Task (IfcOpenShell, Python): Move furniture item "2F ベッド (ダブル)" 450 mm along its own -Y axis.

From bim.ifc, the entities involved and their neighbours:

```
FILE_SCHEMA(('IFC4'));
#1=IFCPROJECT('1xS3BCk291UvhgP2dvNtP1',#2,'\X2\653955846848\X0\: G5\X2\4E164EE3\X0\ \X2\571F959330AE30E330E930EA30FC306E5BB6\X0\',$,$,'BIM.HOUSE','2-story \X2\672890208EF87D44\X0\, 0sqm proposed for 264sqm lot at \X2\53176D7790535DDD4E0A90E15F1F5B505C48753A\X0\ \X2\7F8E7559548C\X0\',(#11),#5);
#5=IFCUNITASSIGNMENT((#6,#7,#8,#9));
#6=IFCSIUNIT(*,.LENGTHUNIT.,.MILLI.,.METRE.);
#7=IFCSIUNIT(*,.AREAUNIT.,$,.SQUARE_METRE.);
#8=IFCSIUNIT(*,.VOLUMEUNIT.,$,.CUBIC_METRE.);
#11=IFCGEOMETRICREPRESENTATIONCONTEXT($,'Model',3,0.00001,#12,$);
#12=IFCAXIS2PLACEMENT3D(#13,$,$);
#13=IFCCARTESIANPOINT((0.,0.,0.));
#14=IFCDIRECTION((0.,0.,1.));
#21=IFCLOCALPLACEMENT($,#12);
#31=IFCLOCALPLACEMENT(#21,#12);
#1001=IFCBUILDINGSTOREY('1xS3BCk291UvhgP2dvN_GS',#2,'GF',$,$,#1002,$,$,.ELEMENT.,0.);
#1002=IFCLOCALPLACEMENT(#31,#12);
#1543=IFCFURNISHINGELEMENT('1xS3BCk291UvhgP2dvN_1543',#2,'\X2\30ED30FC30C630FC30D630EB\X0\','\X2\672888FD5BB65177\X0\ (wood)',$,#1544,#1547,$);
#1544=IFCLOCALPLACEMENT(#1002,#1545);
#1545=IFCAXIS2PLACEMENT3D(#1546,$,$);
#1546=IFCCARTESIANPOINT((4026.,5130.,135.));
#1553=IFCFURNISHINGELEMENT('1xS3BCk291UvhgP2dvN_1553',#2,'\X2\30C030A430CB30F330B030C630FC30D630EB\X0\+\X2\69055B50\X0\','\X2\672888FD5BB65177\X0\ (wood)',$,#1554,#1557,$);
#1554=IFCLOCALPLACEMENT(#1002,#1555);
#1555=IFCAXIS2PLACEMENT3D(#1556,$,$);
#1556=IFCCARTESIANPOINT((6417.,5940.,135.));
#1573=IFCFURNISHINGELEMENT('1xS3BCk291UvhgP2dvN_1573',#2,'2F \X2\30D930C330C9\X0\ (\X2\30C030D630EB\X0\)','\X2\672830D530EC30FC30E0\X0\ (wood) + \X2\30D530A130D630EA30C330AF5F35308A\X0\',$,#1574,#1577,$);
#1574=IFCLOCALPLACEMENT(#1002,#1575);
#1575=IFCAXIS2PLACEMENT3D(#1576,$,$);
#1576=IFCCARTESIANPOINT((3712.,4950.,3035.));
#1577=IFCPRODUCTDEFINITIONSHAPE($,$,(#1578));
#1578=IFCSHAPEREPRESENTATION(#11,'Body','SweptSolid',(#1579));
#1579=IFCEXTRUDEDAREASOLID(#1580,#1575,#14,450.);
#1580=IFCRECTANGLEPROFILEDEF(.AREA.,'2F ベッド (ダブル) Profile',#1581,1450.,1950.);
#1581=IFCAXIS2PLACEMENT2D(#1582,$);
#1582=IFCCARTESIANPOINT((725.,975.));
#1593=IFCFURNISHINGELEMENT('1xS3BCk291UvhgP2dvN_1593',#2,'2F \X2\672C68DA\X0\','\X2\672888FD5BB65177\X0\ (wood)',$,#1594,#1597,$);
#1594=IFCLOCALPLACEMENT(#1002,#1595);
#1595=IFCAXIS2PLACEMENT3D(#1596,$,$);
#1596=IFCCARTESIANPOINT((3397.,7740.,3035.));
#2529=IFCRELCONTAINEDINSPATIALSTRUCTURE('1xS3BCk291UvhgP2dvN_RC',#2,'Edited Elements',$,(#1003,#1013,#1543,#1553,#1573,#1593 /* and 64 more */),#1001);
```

```python
import ifcopenshell
import ifcopenshell.api.geometry
import ifcopenshell.util.placement
import ifcopenshell.util.unit

model = ifcopenshell.open("bim.ifc")
unit_scale = ifcopenshell.util.unit.calculate_unit_scale(model)

item = model.by_id(1573)
matrix = ifcopenshell.util.placement.get_local_placement(item.ObjectPlacement)
matrix[:3, 3] -= matrix[:3, 1] * 0.45 / unit_scale
ifcopenshell.api.geometry.edit_object_placement(model, product=item, matrix=matrix, is_si=False)

print(ifcopenshell.util.placement.get_local_placement(item.ObjectPlacement).round(3) + 0.0)

model.write("bim_v2.ifc")
```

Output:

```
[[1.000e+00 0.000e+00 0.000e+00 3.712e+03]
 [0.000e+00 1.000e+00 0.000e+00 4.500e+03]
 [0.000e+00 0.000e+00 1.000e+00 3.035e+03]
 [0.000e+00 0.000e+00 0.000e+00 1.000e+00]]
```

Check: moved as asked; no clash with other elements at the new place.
